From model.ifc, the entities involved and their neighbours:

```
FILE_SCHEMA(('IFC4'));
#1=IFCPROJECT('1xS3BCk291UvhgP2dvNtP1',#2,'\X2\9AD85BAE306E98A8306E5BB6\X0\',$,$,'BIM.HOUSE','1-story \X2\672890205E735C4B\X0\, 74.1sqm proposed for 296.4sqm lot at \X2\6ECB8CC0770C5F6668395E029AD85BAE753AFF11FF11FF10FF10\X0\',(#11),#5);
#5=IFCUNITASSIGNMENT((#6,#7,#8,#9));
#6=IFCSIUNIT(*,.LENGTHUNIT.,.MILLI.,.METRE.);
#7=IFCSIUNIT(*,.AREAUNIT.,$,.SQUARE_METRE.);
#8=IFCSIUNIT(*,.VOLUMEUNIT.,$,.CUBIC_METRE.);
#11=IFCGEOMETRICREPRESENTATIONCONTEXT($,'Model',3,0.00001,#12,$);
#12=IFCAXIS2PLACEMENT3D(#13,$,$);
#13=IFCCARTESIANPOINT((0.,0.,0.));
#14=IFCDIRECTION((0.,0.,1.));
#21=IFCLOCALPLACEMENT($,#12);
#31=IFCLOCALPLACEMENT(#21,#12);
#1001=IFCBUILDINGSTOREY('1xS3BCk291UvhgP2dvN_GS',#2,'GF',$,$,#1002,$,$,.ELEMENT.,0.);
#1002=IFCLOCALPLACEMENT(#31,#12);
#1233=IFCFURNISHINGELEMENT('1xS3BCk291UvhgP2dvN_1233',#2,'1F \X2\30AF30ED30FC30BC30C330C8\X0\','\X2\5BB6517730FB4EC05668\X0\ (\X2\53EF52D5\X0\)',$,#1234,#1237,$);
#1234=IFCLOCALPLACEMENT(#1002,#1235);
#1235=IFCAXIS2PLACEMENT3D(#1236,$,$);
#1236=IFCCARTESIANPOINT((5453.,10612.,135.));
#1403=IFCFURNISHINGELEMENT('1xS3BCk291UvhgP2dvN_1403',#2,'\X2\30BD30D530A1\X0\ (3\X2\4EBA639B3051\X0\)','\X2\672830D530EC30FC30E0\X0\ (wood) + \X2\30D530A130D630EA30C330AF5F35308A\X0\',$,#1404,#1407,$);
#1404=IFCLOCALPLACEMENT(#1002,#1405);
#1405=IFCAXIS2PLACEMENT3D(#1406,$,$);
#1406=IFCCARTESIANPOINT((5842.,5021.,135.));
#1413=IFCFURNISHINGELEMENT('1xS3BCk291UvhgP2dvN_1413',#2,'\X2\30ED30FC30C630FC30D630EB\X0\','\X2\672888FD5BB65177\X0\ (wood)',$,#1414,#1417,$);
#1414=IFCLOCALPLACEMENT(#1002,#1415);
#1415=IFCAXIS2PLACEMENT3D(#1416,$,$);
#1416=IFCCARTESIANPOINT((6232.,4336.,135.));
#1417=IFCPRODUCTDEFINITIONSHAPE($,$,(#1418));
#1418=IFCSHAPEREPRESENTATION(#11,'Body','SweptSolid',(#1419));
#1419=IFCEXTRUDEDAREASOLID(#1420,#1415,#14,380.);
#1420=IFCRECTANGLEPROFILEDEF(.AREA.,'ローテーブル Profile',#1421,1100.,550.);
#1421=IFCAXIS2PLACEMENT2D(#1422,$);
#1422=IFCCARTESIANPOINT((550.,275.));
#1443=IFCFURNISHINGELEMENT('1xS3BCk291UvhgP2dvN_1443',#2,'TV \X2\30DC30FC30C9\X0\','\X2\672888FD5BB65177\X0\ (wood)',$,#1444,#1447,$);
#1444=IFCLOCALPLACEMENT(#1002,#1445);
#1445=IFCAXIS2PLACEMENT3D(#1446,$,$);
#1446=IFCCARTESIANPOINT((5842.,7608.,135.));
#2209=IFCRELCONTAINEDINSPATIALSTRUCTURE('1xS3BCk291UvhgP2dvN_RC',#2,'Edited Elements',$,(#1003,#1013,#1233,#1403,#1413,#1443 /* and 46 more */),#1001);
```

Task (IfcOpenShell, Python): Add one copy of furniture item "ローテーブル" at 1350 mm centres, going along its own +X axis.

```python
import ifcopenshell
import ifcopenshell.api.geometry
import ifcopenshell.api.root
import ifcopenshell.util.element
import ifcopenshell.util.placement
import ifcopenshell.util.unit

model = ifcopenshell.open("model.ifc")
unit_scale = ifcopenshell.util.unit.calculate_unit_scale(model)


def reuse_history(source, copy):
    """copy_class also copies each property set's owner history, people and application; keep the originals."""
    for rel in copy.IsDefinedBy:
        if rel.is_a("IfcRelDefinesByProperties") and (history := rel.RelatingPropertyDefinition.OwnerHistory):
            rel.RelatingPropertyDefinition.OwnerHistory = source.OwnerHistory
            ifcopenshell.util.element.remove_deep2(model, history)


source = model.by_id(1413)
base = ifcopenshell.util.placement.get_local_placement(source.ObjectPlacement)
step = base[:3, 0] * 1.35 / unit_scale

for i in range(1, 2):
    copy = ifcopenshell.api.root.copy_class(model, product=source)
    copy.Representation = ifcopenshell.util.element.copy_deep(
        model, source.Representation, exclude=["IfcGeometricRepresentationContext", "IfcRepresentationMap"]
    )
    reuse_history(source, copy)
    matrix = base.copy()
    matrix[:3, 3] += i * step
    print("added at", matrix[:3, 3].round(3) + 0.0)
    ifcopenshell.api.geometry.edit_object_placement(model, product=copy, matrix=matrix, is_si=False)

model.write("model_updated.ifc")
```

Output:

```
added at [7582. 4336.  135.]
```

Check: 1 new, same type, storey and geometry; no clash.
